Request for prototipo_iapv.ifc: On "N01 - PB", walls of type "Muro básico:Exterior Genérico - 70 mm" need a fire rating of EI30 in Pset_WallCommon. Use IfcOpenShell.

First a look at what the model holds.

```python
import ifcopenshell
import ifcopenshell.util.element

model = ifcopenshell.open("prototipo_iapv.ifc")
print(model.schema)
storey = next(s for s in model.by_type("IfcBuildingStorey") if s.Name == "N01 - PB")
walls = [e for e in ifcopenshell.util.element.get_decomposition(storey) if e.is_a("IfcWall")]
seen = {}
for e in walls:
    element_type = ifcopenshell.util.element.get_type(e)
    key = (element_type.Name if element_type != e and element_type else None, ifcopenshell.util.element.get_pset(e, "Pset_WallCommon", "FireRating"))
    seen[key] = seen.get(key, 0) + 1
for (name, value), count in sorted(seen.items(), key=str):
    print(count, "x", name, "|", value)
```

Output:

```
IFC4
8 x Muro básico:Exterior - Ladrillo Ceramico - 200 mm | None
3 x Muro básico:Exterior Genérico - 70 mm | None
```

```python
import ifcopenshell
import ifcopenshell.api.pset
import ifcopenshell.util.element

model = ifcopenshell.open("prototipo_iapv.ifc")

storey = next(s for s in model.by_type("IfcBuildingStorey") if s.Name == "N01 - PB")
walls = [e for e in ifcopenshell.util.element.get_decomposition(storey) if e.is_a("IfcWall")]

count = 0
for e in walls:
    element_type = ifcopenshell.util.element.get_type(e)
    if element_type in (None, e) or element_type.Name != "Muro básico:Exterior Genérico - 70 mm":
        continue
    # add_pset returns the element's existing set when there is one.
    pset = ifcopenshell.api.pset.add_pset(model, product=e, name="Pset_WallCommon")
    ifcopenshell.api.pset.edit_pset(model, pset=pset, properties={"FireRating": "EI30"})
    count += 1

print(count, "walls updated")

model.write("prototipo_iapv-out.ifc")
```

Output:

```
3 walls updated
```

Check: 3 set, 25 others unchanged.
